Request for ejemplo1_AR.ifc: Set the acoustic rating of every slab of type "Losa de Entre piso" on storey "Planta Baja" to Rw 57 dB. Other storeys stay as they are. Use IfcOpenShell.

First a look at what the model holds.

```python
import ifcopenshell
import ifcopenshell.util.element

model = ifcopenshell.open("ejemplo1_AR.ifc")
print(model.schema)
storey = next(s for s in model.by_type("IfcBuildingStorey") if s.Name == "Planta Baja")
slabs = [e for e in ifcopenshell.util.element.get_decomposition(storey) if e.is_a("IfcSlab")]
seen = {}
for e in slabs:
    element_type = ifcopenshell.util.element.get_type(e)
    key = (element_type.Name if element_type != e and element_type else None, ifcopenshell.util.element.get_pset(e, "Pset_SlabCommon", "AcousticRating"))
    seen[key] = seen.get(key, 0) + 1
for (name, value), count in sorted(seen.items(), key=str):
    print(count, "x", name, "|", value)
```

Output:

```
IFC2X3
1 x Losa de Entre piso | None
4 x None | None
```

```python
import ifcopenshell
import ifcopenshell.api.pset
import ifcopenshell.util.element

model = ifcopenshell.open("ejemplo1_AR.ifc")

storey = next(s for s in model.by_type("IfcBuildingStorey") if s.Name == "Planta Baja")
slabs = [e for e in ifcopenshell.util.element.get_decomposition(storey) if e.is_a("IfcSlab")]

count = 0
for e in slabs:
    element_type = ifcopenshell.util.element.get_type(e)
    if element_type in (None, e) or element_type.Name != "Losa de Entre piso":
        continue
    # add_pset returns the element's existing set when there is one.
    pset = ifcopenshell.api.pset.add_pset(model, product=e, name="Pset_SlabCommon")
    ifcopenshell.api.pset.edit_pset(model, pset=pset, properties={"AcousticRating": "Rw 57 dB"})
    count += 1

print(count, "slabs updated")

model.write("ejemplo1_AR_updated.ifc")
```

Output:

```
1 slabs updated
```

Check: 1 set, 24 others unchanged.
